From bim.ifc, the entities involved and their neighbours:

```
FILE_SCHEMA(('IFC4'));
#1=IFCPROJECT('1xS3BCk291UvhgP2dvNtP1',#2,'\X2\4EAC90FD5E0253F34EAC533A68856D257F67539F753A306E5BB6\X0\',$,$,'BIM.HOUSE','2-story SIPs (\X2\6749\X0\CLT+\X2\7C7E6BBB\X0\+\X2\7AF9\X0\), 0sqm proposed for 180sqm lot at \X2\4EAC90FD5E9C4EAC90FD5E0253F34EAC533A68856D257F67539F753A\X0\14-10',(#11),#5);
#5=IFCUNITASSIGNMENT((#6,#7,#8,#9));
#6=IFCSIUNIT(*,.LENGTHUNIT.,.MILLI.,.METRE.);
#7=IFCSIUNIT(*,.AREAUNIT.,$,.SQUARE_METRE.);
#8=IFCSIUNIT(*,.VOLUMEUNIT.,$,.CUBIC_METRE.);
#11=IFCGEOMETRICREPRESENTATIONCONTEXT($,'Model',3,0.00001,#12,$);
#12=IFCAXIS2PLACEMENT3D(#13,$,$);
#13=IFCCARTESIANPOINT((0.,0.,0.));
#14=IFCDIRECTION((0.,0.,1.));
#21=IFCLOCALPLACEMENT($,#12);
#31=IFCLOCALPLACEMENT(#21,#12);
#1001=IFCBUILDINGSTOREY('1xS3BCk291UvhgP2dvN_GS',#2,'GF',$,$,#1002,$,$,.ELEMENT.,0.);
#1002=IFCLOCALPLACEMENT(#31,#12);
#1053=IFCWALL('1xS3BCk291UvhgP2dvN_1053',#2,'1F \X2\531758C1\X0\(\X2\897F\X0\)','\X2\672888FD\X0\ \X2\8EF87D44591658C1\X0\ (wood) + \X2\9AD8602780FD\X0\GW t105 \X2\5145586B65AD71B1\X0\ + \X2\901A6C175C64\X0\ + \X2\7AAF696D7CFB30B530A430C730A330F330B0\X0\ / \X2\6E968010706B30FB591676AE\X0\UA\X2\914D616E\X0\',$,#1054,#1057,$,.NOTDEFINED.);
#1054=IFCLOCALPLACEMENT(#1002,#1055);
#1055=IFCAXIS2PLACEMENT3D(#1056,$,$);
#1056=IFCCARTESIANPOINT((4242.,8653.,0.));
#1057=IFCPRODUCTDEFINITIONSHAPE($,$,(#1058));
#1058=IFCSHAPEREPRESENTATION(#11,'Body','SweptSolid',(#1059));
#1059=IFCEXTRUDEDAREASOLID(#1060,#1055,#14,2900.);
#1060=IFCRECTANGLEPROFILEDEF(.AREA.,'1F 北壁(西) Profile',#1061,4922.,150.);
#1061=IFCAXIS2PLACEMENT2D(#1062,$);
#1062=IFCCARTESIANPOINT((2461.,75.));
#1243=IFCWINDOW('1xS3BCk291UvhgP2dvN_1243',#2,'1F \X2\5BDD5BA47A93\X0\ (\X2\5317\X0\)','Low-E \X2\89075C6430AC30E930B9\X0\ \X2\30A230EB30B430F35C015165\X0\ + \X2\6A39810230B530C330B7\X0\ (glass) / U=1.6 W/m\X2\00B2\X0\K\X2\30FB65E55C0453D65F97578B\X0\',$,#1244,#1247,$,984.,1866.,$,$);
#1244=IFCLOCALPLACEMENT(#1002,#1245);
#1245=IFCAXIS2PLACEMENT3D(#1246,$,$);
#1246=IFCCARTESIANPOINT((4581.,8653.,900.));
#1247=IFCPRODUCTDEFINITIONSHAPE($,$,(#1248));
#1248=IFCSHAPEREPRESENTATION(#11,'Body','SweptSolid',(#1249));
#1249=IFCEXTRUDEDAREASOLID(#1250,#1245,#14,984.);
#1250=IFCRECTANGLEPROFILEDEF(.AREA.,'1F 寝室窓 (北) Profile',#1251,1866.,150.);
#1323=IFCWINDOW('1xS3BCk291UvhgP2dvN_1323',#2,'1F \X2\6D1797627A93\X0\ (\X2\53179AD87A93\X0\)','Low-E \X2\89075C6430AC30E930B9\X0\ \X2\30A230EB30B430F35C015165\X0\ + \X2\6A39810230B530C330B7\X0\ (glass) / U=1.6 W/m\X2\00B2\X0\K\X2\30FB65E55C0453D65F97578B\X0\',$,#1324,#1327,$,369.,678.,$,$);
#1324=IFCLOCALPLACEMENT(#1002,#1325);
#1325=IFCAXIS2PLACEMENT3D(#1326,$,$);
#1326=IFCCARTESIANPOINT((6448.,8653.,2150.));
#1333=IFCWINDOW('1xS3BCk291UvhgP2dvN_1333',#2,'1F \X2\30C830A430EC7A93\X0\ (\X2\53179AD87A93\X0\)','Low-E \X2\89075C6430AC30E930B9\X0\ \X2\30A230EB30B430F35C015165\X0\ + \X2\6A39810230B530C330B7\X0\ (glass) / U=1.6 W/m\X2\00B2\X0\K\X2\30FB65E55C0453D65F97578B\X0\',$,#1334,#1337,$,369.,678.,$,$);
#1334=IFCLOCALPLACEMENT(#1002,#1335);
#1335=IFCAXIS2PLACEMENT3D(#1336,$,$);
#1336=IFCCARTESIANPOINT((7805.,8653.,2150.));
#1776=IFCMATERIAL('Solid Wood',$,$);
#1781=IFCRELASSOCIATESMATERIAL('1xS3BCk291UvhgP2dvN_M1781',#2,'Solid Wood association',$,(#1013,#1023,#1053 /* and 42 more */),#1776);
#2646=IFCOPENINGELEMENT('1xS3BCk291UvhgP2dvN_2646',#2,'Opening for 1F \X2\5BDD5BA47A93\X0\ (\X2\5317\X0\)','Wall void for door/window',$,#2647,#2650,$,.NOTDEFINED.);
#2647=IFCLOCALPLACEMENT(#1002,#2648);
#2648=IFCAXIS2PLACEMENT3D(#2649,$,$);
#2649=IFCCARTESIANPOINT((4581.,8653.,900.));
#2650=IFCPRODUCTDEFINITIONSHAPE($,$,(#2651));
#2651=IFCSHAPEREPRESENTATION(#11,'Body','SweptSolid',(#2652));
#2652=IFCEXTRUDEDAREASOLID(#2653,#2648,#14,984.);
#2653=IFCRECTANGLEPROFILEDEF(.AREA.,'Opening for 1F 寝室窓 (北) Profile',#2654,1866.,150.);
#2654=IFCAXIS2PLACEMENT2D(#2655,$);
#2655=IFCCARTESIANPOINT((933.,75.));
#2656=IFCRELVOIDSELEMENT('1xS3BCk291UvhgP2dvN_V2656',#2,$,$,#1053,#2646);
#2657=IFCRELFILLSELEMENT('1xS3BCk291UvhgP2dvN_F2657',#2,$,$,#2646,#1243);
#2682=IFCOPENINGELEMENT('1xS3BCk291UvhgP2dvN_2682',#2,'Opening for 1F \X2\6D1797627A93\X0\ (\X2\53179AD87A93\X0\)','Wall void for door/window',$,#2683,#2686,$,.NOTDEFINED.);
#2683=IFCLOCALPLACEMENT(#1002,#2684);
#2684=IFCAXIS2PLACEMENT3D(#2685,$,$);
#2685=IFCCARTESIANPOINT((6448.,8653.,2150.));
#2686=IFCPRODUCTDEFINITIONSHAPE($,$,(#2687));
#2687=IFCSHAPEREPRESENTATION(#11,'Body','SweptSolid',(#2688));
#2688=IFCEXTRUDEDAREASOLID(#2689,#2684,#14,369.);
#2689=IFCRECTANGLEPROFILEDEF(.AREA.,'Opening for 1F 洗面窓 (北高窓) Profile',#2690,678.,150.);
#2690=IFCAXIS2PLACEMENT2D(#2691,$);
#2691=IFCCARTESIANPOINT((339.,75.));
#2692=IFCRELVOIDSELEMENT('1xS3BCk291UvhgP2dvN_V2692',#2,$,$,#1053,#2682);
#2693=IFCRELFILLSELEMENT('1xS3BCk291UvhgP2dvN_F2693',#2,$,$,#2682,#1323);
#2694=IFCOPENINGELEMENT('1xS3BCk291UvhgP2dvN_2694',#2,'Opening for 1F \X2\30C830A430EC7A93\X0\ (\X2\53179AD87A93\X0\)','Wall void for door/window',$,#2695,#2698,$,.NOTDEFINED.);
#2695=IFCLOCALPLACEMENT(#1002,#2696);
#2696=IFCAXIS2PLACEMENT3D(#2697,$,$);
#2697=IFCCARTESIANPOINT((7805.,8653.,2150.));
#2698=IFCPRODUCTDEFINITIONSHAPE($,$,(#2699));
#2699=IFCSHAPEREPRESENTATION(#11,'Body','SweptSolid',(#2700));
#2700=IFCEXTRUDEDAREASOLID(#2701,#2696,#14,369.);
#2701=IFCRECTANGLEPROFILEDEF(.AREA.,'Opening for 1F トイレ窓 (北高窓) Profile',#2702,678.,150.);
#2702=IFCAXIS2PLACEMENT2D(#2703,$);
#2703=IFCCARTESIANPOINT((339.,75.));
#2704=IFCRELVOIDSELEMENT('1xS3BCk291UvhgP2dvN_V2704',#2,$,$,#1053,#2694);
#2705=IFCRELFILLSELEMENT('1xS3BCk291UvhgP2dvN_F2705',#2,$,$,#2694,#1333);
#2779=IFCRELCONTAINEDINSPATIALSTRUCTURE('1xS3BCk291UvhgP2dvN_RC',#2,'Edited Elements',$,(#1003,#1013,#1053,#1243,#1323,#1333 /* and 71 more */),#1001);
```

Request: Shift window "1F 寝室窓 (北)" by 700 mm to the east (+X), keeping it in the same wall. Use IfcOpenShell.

```python
import ifcopenshell
import ifcopenshell.api.geometry
import ifcopenshell.util.placement

model = ifcopenshell.open("bim.ifc")

window = model.by_guid("1xS3BCk291UvhgP2dvN_1243")
opening = window.FillsVoids[0].RelatingOpeningElement
wall = opening.VoidsElements[0].RelatingBuildingElement

wall_matrix = ifcopenshell.util.placement.get_local_placement(wall.ObjectPlacement)
shift = wall_matrix[:3, 0] * 700.0
before = ifcopenshell.util.placement.get_local_placement(window.ObjectPlacement)[:3, 3].copy()

# The window is not placed relative to its opening, so move both.
for product in (opening, window):
    matrix = ifcopenshell.util.placement.get_local_placement(product.ObjectPlacement)
    matrix[:3, 3] += shift
    ifcopenshell.api.geometry.edit_object_placement(model, product=product, matrix=matrix, is_si=False)

after = ifcopenshell.util.placement.get_local_placement(window.ObjectPlacement)[:3, 3]
print("window moved by", (after - before).round(3) + 0.0)

model.write("bim-out.ifc")
```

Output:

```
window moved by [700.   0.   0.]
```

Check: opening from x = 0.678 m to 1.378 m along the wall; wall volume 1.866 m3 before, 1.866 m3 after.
